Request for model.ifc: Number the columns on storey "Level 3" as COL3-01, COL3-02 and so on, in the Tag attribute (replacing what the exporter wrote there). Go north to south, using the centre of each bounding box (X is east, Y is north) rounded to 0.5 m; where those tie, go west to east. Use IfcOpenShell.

First a look at what the model holds.

```python
import ifcopenshell
import ifcopenshell.util.element
import ifcopenshell.util.placement

model = ifcopenshell.open("model.ifc")
print(model.schema)
storey = next(s for s in model.by_type("IfcBuildingStorey") if s.Name == "Level 3")
columns = [e for e in ifcopenshell.util.element.get_decomposition(storey) if e.is_a("IfcColumn")]
for e in sorted(columns, key=lambda e: e.id()):
    origin = ifcopenshell.util.placement.get_local_placement(e.ObjectPlacement)[:3, 3]
    print(e.id(), e.Tag, e.Name, origin.round(2) + 0.0, sep=" | ")
```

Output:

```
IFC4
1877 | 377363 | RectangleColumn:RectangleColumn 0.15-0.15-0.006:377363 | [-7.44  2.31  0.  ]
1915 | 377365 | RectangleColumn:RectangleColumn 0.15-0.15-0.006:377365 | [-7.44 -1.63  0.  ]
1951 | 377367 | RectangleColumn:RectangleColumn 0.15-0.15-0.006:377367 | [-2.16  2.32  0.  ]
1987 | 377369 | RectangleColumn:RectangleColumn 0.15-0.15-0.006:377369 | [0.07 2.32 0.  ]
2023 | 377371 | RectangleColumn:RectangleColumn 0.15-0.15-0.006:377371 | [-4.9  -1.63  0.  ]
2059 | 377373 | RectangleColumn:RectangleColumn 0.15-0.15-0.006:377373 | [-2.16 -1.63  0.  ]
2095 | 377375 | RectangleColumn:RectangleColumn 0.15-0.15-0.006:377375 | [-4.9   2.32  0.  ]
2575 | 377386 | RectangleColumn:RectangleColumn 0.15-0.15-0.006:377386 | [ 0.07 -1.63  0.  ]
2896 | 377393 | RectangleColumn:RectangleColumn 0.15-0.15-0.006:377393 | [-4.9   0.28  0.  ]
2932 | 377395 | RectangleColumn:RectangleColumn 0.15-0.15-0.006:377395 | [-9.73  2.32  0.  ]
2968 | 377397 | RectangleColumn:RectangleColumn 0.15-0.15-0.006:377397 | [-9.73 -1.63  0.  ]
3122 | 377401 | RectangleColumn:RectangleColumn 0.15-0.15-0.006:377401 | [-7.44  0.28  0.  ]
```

```python
import ifcopenshell
import ifcopenshell.geom
import ifcopenshell.util.element
import ifcopenshell.util.shape

model = ifcopenshell.open("model.ifc")
settings = ifcopenshell.geom.settings()
settings.set("use-world-coords", True)


def centre(element):
    shape = ifcopenshell.geom.create_shape(settings, element)
    return ifcopenshell.util.shape.get_bbox_centroid(shape.geometry)


storey = next(s for s in model.by_type("IfcBuildingStorey") if s.Name == "Level 3")
columns = [e for e in ifcopenshell.util.element.get_decomposition(storey) if e.is_a("IfcColumn")]

# Insertion points can sit at a corner or the storey origin, so sort by the geometry (in metres).
centres = {e: centre(e) for e in columns}
columns.sort(key=lambda e: (-round(centres[e][1] / 0.5), centres[e][0]))

for i, e in enumerate(columns, start=1):
    number = f"COL3-{i:02d}"
    e.Tag = number
    print(e.id(), number)

model.write("model-out.ifc")
```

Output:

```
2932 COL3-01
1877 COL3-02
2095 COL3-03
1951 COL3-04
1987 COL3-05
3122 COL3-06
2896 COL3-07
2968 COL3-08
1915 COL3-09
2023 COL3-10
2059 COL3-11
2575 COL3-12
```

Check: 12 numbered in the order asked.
